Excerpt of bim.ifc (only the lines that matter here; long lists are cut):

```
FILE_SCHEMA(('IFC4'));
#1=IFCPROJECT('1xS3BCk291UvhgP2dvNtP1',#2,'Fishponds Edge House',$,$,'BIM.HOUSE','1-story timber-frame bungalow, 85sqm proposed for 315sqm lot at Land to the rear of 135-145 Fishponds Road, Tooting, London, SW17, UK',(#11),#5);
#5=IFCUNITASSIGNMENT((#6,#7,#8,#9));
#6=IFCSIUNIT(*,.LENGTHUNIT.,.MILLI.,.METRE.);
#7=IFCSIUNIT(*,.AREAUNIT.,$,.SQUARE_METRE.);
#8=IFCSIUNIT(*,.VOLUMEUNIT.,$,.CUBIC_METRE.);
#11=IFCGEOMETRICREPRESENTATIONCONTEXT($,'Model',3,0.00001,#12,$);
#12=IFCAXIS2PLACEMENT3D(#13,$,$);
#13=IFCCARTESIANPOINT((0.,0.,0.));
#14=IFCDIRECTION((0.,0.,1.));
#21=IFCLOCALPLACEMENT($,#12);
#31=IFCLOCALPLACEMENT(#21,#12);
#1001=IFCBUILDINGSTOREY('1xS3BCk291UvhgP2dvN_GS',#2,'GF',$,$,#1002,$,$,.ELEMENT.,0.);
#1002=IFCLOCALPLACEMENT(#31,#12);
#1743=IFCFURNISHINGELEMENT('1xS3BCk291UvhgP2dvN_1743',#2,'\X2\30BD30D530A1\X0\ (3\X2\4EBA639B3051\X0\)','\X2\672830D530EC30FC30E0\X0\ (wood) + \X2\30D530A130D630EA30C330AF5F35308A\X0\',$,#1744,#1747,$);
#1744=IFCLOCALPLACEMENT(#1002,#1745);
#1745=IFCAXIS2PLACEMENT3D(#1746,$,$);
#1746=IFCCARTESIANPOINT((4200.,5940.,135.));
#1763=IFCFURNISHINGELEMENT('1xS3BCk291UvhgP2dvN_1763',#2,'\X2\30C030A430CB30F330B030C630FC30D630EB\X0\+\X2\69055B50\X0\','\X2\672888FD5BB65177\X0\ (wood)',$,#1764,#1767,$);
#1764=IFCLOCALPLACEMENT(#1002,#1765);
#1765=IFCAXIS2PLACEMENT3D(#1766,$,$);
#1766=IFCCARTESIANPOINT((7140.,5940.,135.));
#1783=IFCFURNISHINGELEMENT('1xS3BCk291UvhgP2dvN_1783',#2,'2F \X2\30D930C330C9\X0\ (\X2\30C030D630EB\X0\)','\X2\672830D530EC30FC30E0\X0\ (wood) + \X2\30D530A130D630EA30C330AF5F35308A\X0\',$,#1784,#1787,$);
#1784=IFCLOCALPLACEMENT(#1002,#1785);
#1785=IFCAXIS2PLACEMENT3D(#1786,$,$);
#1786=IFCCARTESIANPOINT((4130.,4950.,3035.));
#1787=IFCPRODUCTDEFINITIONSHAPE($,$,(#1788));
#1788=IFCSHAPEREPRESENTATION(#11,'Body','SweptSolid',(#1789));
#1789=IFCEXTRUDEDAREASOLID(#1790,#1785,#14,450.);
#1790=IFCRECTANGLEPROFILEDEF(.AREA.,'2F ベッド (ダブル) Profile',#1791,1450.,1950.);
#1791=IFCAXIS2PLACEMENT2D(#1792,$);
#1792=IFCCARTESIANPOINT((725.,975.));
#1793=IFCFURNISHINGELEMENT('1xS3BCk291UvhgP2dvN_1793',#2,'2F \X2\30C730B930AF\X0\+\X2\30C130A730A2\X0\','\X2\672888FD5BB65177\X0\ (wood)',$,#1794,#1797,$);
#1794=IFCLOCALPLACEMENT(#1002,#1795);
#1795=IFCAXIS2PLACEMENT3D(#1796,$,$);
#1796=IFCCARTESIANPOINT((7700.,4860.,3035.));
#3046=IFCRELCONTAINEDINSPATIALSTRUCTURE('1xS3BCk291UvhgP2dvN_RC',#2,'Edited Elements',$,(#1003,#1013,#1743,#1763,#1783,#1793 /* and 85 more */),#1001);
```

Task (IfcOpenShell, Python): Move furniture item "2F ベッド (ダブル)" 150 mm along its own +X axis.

```python
import ifcopenshell
import ifcopenshell.api.geometry
import ifcopenshell.util.placement

model = ifcopenshell.open("bim.ifc")

item = model.by_guid("1xS3BCk291UvhgP2dvN_1783")
matrix = ifcopenshell.util.placement.get_local_placement(item.ObjectPlacement)
matrix[:3, 3] += matrix[:3, 0] * 150.0
ifcopenshell.api.geometry.edit_object_placement(model, product=item, matrix=matrix, is_si=False)

print(ifcopenshell.util.placement.get_local_placement(item.ObjectPlacement).round(3) + 0.0)

model.write("bim_updated.ifc")
```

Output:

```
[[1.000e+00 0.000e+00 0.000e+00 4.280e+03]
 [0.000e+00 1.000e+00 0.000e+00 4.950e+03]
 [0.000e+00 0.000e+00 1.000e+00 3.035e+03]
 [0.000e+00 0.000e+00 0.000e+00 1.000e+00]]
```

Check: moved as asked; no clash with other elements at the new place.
